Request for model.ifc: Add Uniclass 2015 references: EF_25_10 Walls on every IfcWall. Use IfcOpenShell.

First a look at what the model holds.

```python
import ifcopenshell

model = ifcopenshell.open("model.ifc")
print(model.schema)
print("classifications:", [c.Name for c in model.by_type("IfcClassification")])
for ifc_class in ("IfcDoor", "IfcRoof", "IfcStair", "IfcWall", "IfcWindow"):
    print(ifc_class, len(model.by_type(ifc_class)))
```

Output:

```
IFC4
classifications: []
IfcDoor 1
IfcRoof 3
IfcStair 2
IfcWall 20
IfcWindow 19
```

```python
import ifcopenshell
import ifcopenshell.api.classification

model = ifcopenshell.open("model.ifc")

system = ifcopenshell.api.classification.add_classification(model, classification="Uniclass 2015")

codes = {
    "IfcWall": ("EF_25_10", "Walls"),
}
for ifc_class, (code, name) in codes.items():
    products = model.by_type(ifc_class)
    ifcopenshell.api.classification.add_reference(
        model, products=products, classification=system, identification=code, name=name
    )
    print(code, len(products))

model.write("model_rev.ifc")
```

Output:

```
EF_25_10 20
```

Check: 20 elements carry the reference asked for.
